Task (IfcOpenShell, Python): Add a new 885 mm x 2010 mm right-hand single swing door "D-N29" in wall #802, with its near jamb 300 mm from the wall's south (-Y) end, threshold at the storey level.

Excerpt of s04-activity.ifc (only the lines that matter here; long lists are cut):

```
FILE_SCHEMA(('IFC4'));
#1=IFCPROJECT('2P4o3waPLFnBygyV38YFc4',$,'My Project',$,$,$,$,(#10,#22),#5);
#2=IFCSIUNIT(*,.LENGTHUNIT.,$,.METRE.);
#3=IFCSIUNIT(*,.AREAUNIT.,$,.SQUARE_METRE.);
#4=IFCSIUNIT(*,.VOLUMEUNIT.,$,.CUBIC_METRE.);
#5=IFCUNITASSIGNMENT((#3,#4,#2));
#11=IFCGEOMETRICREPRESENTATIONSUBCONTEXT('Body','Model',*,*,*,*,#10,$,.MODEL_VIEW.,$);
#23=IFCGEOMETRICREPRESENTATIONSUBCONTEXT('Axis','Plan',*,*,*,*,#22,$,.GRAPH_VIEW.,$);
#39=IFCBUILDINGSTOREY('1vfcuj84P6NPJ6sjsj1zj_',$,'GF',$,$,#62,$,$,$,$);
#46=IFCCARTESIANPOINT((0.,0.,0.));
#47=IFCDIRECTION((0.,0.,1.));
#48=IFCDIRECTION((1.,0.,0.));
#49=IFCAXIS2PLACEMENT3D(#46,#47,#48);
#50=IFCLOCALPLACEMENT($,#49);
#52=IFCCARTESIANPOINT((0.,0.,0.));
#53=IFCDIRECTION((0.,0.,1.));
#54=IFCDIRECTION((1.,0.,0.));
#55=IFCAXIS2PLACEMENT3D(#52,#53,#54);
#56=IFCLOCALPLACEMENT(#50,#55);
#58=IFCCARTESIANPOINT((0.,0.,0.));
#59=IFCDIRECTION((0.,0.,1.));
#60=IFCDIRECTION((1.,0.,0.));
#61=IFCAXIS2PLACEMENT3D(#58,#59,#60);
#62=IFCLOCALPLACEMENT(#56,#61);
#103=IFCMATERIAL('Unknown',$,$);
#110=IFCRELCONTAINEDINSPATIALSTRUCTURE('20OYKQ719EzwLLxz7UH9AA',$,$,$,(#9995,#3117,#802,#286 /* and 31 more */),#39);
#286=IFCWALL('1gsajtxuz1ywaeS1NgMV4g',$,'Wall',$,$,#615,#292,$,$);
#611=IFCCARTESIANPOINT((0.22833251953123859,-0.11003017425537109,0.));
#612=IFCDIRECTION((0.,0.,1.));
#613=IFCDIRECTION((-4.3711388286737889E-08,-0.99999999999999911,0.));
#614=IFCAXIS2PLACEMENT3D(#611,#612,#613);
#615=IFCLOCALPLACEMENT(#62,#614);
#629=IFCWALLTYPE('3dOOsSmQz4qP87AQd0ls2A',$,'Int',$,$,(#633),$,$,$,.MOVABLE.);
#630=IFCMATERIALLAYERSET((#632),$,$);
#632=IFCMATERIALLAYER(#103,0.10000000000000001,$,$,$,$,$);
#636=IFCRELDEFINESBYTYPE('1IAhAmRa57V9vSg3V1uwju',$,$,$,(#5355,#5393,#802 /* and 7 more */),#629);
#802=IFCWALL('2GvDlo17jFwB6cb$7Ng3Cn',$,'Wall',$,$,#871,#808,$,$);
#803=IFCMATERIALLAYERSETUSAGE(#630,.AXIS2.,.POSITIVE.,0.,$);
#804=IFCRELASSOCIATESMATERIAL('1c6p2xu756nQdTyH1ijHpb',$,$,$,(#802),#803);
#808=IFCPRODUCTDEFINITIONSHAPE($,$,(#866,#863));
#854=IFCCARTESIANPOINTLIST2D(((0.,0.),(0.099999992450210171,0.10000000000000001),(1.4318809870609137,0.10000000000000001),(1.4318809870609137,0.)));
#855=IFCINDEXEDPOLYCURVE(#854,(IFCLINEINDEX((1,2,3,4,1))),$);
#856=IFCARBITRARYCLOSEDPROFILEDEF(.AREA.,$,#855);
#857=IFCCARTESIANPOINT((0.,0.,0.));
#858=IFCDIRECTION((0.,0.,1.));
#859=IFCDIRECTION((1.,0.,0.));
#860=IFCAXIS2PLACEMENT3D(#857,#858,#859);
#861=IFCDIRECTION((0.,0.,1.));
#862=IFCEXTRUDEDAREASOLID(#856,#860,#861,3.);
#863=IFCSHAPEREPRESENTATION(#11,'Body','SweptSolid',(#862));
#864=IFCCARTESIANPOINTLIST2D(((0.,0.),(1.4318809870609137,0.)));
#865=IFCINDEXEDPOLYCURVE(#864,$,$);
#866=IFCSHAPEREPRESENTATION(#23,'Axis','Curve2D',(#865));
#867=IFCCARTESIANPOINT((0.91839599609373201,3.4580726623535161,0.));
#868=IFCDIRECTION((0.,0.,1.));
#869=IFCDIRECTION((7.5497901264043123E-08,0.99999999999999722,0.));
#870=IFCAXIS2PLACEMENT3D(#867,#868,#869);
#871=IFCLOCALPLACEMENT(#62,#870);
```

```python
import numpy as np
import ifcopenshell
import ifcopenshell.api.feature
import ifcopenshell.api.geometry
import ifcopenshell.api.root
import ifcopenshell.api.spatial
import ifcopenshell.geom
import ifcopenshell.util.element
import ifcopenshell.util.placement
import ifcopenshell.util.representation
import ifcopenshell.util.shape
import ifcopenshell.util.unit

model = ifcopenshell.open("s04-activity.ifc")
unit_scale = ifcopenshell.util.unit.calculate_unit_scale(model)
settings = ifcopenshell.geom.settings()


def volume(element):
    """Net volume in cubic metres, openings subtracted."""
    shape = ifcopenshell.geom.create_shape(settings, element)
    return ifcopenshell.util.shape.get_volume(shape.geometry)


wall = model.by_guid("2GvDlo17jFwB6cb$7Ng3Cn")
storey = ifcopenshell.util.element.get_container(wall, ifc_class="IfcBuildingStorey")
context = ifcopenshell.util.representation.get_context(model, "Model", "Body", "MODEL_VIEW")
before = volume(wall)

width, height, from_end, sill = 0.885, 2.01, 0.3, 0.0  # metres

# The wall runs along its own X axis, and the end named is its -X end.
wall_shape = ifcopenshell.geom.create_shape(settings, wall)
x, y, z = ifcopenshell.util.shape.get_vertices(wall_shape.geometry).T
start = x.min() + from_end
face, thickness = float(y.min()), float(y.max() - y.min())
wall_matrix = ifcopenshell.util.placement.get_local_placement(wall.ObjectPlacement)
level = ifcopenshell.util.placement.get_local_placement(storey.ObjectPlacement)[2, 3]


def in_wall(x, y):
    """Placement at x, y metres in the wall's axes, at sill height."""
    matrix = wall_matrix.copy()
    matrix[:, 3] = wall_matrix @ np.array([x / unit_scale, y / unit_scale, 0.0, 1.0])
    matrix[2, 3] = level + sill / unit_scale
    return matrix


# Opening: a box that overshoots both wall faces by 50 mm.
opening = ifcopenshell.api.root.create_entity(model, ifc_class="IfcOpeningElement", predefined_type="OPENING")
box = ifcopenshell.api.geometry.add_wall_representation(
    model, context=context, length=width, height=height, thickness=thickness + 0.1
)
ifcopenshell.api.geometry.assign_representation(model, product=opening, representation=box)
ifcopenshell.api.geometry.edit_object_placement(model, product=opening, matrix=in_wall(start, face - 0.05), is_si=False)
ifcopenshell.api.feature.add_feature(model, feature=opening, element=wall)

door = ifcopenshell.api.root.create_entity(model, ifc_class="IfcDoor", name="D-N29", predefined_type="DOOR")
door.OverallWidth, door.OverallHeight = width / unit_scale, height / unit_scale
door.OperationType = "SINGLE_SWING_RIGHT"
body = ifcopenshell.api.geometry.add_door_representation(
    model,
    context=context,
    overall_width=door.OverallWidth,
    overall_height=door.OverallHeight,
    operation_type="SINGLE_SWING_RIGHT",
    lining_properties={"LiningDepth": thickness / unit_scale, "ThresholdDepth": thickness / unit_scale},
)
ifcopenshell.api.geometry.assign_representation(model, product=door, representation=body)
ifcopenshell.api.spatial.assign_container(model, products=[door], relating_structure=storey)
ifcopenshell.api.feature.add_filling(model, opening=opening, element=door)

# The lining spans the wall, so the door starts at the wall face.
ifcopenshell.api.geometry.edit_object_placement(model, product=door, matrix=in_wall(start, face), is_si=False)

after = volume(wall)

print(f"wall volume {before:.3f} -> {after:.3f} m3")

model.write("s04-activity_v2.ifc")
```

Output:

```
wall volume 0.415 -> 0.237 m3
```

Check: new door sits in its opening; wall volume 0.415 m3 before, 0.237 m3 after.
